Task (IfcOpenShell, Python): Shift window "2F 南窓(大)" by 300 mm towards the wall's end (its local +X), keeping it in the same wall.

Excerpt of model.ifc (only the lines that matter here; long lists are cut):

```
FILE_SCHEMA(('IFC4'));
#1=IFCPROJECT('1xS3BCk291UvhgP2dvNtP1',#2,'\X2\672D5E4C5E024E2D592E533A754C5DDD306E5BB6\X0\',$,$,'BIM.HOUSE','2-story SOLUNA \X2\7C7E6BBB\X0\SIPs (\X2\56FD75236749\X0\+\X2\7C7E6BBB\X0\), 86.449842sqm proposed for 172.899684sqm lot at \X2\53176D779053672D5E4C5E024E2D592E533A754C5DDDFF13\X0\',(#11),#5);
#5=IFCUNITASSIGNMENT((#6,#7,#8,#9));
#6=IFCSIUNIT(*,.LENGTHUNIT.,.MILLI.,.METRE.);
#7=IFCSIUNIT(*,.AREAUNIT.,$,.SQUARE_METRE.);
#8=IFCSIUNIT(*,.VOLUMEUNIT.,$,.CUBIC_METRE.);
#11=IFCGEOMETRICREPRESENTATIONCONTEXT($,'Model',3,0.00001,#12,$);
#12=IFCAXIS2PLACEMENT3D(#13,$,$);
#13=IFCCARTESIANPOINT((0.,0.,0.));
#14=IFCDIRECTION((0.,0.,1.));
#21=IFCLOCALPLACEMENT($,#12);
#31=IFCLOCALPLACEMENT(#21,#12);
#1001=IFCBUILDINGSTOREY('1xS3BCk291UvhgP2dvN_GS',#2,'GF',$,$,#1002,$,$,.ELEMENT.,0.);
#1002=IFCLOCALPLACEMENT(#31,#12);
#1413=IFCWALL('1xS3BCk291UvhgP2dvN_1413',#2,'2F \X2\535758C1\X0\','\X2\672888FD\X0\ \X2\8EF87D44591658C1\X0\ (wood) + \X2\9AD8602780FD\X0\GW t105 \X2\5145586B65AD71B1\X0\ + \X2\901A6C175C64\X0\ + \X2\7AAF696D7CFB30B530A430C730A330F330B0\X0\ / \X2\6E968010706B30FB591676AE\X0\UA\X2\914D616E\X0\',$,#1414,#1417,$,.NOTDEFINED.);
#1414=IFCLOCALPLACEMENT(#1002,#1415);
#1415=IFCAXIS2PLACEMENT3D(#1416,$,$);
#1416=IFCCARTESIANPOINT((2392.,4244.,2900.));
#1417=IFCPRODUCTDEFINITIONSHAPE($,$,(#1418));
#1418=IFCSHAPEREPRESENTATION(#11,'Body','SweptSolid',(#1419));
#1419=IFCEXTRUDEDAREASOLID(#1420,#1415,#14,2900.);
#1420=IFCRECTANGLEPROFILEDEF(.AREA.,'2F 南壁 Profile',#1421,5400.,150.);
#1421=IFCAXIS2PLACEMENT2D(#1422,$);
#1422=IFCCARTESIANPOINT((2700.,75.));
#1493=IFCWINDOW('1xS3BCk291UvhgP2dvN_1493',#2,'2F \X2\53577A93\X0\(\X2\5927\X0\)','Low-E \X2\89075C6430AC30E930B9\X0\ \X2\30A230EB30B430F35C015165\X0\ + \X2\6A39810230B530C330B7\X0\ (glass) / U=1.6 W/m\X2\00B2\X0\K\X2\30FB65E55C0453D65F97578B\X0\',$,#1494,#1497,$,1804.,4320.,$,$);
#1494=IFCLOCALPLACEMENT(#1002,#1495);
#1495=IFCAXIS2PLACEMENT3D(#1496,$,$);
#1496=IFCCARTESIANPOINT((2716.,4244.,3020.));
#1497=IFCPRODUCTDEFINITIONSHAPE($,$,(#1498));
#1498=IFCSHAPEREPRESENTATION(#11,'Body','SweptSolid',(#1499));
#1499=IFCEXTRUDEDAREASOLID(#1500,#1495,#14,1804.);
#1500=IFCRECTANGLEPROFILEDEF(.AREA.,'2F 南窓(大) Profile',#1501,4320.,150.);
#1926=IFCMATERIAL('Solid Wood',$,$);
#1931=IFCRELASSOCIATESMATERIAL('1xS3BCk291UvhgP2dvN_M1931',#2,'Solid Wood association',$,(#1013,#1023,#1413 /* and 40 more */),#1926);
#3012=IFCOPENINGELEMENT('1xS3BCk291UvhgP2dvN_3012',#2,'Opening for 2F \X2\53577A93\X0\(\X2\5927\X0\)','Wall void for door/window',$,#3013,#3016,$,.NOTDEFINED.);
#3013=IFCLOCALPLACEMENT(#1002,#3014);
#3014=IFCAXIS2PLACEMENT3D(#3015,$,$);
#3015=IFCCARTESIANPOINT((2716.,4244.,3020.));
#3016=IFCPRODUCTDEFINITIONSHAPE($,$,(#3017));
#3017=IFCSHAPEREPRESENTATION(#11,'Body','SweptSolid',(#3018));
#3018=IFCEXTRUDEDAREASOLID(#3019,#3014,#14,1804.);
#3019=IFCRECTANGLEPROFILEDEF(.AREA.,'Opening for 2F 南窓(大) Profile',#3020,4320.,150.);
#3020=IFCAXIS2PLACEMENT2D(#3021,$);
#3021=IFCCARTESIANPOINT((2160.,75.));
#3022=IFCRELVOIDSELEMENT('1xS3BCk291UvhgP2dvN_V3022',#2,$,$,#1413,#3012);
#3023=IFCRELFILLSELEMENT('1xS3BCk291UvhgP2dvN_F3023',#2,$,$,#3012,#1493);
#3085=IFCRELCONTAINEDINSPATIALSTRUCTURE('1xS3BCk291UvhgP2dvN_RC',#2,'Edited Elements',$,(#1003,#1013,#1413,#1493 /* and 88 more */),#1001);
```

```python
import ifcopenshell
import ifcopenshell.api.geometry
import ifcopenshell.util.placement
import ifcopenshell.util.unit

model = ifcopenshell.open("model.ifc")
unit_scale = ifcopenshell.util.unit.calculate_unit_scale(model)

window = model.by_guid("1xS3BCk291UvhgP2dvN_1493")
opening = window.FillsVoids[0].RelatingOpeningElement
wall = opening.VoidsElements[0].RelatingBuildingElement

wall_matrix = ifcopenshell.util.placement.get_local_placement(wall.ObjectPlacement)
shift = wall_matrix[:3, 0] * 0.3 / unit_scale
before = ifcopenshell.util.placement.get_local_placement(window.ObjectPlacement)[:3, 3].copy()

# The window is not placed relative to its opening, so move both.
for product in (opening, window):
    matrix = ifcopenshell.util.placement.get_local_placement(product.ObjectPlacement)
    matrix[:3, 3] += shift
    ifcopenshell.api.geometry.edit_object_placement(model, product=product, matrix=matrix, is_si=False)

after = ifcopenshell.util.placement.get_local_placement(window.ObjectPlacement)[:3, 3]
print("window moved by", (after - before).round(3) + 0.0)

model.write("model_v2.ifc")
```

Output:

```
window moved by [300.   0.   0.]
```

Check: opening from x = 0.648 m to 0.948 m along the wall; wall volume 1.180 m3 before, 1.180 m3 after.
